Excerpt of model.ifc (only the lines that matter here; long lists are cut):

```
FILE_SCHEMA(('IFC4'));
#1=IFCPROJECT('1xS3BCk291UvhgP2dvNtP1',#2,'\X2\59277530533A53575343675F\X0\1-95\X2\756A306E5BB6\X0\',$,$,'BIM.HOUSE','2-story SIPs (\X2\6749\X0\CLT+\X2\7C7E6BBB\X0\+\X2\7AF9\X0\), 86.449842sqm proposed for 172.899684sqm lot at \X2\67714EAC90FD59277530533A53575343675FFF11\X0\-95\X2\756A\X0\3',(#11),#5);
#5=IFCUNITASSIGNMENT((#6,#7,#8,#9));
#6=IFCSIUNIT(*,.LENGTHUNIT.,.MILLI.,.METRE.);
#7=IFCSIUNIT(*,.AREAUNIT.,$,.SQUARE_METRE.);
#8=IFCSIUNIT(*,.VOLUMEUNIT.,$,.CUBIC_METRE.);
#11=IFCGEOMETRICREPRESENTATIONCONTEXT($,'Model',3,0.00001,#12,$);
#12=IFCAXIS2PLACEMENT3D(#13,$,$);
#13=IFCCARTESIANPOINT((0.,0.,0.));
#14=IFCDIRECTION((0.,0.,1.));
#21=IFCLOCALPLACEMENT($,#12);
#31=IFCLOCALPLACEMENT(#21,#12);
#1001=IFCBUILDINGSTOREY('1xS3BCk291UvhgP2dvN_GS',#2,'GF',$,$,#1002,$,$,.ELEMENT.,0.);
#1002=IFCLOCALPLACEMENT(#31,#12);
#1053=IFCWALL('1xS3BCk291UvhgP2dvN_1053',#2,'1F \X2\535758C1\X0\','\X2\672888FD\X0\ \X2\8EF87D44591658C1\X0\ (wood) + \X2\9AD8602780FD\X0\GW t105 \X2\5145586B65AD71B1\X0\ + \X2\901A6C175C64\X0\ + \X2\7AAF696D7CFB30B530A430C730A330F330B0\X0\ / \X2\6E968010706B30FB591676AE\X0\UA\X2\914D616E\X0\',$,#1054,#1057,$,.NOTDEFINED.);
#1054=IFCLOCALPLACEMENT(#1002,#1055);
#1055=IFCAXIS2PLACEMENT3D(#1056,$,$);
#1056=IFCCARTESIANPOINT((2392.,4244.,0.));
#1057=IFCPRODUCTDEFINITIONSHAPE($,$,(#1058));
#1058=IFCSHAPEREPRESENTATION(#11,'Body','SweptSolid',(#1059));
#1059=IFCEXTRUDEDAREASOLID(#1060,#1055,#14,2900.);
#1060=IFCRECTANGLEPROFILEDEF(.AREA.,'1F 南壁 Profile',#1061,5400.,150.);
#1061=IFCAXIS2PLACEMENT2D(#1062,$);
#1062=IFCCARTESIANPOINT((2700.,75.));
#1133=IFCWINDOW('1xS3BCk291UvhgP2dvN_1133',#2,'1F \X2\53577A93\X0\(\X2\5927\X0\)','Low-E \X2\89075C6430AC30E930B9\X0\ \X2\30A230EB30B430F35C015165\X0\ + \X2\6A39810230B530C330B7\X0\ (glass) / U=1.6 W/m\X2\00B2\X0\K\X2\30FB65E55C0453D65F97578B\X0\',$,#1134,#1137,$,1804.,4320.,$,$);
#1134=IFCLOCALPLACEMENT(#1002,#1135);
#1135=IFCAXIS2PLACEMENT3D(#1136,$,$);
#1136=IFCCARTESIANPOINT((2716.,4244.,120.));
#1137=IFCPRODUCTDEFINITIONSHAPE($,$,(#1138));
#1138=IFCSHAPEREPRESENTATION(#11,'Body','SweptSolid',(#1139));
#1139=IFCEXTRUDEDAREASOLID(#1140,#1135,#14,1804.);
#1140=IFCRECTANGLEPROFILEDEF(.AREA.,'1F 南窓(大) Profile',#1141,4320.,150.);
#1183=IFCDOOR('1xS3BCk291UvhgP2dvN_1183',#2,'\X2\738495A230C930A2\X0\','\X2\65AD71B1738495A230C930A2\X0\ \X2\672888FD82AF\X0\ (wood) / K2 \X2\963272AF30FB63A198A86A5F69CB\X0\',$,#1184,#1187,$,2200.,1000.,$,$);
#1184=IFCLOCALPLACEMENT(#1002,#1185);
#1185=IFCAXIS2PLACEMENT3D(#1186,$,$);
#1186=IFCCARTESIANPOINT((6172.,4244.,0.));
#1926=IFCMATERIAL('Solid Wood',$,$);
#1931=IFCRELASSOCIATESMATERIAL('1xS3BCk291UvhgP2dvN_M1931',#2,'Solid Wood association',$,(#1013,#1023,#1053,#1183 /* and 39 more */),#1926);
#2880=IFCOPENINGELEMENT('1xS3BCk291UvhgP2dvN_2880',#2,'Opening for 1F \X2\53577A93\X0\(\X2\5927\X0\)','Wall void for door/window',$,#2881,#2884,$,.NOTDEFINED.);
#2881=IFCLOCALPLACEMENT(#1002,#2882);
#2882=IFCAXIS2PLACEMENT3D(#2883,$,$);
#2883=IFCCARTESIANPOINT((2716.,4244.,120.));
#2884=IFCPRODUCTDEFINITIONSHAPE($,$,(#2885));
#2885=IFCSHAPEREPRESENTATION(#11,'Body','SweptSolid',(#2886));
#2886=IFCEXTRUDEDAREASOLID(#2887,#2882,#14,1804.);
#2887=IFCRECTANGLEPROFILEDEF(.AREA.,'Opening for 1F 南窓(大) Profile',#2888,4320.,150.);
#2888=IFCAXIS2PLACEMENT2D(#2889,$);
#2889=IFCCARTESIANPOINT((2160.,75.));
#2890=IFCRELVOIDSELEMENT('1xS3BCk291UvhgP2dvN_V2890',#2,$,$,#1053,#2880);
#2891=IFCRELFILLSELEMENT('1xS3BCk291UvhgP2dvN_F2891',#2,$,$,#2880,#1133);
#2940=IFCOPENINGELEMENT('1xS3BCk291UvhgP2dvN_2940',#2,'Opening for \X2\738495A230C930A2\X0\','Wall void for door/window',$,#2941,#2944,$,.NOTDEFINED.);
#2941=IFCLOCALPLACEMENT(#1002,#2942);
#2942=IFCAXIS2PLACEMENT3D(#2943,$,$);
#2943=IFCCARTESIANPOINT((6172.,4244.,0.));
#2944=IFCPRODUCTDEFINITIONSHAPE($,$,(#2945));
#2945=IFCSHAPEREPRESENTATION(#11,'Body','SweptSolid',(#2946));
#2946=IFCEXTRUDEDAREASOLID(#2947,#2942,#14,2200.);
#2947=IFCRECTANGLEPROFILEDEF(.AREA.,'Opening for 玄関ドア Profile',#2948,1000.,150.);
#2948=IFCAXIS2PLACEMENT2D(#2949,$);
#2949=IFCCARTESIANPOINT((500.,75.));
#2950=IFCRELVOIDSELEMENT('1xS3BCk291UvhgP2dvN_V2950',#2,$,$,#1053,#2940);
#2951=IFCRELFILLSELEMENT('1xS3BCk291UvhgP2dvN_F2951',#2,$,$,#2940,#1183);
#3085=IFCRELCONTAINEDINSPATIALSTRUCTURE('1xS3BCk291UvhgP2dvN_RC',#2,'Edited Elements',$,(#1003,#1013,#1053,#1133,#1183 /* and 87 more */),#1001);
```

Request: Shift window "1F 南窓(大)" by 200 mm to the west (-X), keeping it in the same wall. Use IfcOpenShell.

```python
import ifcopenshell
import ifcopenshell.api.geometry
import ifcopenshell.util.placement

model = ifcopenshell.open("model.ifc")

window = model.by_guid("1xS3BCk291UvhgP2dvN_1133")
opening = window.FillsVoids[0].RelatingOpeningElement
wall = opening.VoidsElements[0].RelatingBuildingElement

wall_matrix = ifcopenshell.util.placement.get_local_placement(wall.ObjectPlacement)
shift = wall_matrix[:3, 0] * -200.0
before = ifcopenshell.util.placement.get_local_placement(window.ObjectPlacement)[:3, 3].copy()

# The window is not placed relative to its opening, so move both.
for product in (opening, window):
    matrix = ifcopenshell.util.placement.get_local_placement(product.ObjectPlacement)
    matrix[:3, 3] += shift
    ifcopenshell.api.geometry.edit_object_placement(model, product=product, matrix=matrix, is_si=False)

after = ifcopenshell.util.placement.get_local_placement(window.ObjectPlacement)[:3, 3]
print("window moved by", (after - before).round(3) + 0.0)

model.write("model_v2.ifc")
```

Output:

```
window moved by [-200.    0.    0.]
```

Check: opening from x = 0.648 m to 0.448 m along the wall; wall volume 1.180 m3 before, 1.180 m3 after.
